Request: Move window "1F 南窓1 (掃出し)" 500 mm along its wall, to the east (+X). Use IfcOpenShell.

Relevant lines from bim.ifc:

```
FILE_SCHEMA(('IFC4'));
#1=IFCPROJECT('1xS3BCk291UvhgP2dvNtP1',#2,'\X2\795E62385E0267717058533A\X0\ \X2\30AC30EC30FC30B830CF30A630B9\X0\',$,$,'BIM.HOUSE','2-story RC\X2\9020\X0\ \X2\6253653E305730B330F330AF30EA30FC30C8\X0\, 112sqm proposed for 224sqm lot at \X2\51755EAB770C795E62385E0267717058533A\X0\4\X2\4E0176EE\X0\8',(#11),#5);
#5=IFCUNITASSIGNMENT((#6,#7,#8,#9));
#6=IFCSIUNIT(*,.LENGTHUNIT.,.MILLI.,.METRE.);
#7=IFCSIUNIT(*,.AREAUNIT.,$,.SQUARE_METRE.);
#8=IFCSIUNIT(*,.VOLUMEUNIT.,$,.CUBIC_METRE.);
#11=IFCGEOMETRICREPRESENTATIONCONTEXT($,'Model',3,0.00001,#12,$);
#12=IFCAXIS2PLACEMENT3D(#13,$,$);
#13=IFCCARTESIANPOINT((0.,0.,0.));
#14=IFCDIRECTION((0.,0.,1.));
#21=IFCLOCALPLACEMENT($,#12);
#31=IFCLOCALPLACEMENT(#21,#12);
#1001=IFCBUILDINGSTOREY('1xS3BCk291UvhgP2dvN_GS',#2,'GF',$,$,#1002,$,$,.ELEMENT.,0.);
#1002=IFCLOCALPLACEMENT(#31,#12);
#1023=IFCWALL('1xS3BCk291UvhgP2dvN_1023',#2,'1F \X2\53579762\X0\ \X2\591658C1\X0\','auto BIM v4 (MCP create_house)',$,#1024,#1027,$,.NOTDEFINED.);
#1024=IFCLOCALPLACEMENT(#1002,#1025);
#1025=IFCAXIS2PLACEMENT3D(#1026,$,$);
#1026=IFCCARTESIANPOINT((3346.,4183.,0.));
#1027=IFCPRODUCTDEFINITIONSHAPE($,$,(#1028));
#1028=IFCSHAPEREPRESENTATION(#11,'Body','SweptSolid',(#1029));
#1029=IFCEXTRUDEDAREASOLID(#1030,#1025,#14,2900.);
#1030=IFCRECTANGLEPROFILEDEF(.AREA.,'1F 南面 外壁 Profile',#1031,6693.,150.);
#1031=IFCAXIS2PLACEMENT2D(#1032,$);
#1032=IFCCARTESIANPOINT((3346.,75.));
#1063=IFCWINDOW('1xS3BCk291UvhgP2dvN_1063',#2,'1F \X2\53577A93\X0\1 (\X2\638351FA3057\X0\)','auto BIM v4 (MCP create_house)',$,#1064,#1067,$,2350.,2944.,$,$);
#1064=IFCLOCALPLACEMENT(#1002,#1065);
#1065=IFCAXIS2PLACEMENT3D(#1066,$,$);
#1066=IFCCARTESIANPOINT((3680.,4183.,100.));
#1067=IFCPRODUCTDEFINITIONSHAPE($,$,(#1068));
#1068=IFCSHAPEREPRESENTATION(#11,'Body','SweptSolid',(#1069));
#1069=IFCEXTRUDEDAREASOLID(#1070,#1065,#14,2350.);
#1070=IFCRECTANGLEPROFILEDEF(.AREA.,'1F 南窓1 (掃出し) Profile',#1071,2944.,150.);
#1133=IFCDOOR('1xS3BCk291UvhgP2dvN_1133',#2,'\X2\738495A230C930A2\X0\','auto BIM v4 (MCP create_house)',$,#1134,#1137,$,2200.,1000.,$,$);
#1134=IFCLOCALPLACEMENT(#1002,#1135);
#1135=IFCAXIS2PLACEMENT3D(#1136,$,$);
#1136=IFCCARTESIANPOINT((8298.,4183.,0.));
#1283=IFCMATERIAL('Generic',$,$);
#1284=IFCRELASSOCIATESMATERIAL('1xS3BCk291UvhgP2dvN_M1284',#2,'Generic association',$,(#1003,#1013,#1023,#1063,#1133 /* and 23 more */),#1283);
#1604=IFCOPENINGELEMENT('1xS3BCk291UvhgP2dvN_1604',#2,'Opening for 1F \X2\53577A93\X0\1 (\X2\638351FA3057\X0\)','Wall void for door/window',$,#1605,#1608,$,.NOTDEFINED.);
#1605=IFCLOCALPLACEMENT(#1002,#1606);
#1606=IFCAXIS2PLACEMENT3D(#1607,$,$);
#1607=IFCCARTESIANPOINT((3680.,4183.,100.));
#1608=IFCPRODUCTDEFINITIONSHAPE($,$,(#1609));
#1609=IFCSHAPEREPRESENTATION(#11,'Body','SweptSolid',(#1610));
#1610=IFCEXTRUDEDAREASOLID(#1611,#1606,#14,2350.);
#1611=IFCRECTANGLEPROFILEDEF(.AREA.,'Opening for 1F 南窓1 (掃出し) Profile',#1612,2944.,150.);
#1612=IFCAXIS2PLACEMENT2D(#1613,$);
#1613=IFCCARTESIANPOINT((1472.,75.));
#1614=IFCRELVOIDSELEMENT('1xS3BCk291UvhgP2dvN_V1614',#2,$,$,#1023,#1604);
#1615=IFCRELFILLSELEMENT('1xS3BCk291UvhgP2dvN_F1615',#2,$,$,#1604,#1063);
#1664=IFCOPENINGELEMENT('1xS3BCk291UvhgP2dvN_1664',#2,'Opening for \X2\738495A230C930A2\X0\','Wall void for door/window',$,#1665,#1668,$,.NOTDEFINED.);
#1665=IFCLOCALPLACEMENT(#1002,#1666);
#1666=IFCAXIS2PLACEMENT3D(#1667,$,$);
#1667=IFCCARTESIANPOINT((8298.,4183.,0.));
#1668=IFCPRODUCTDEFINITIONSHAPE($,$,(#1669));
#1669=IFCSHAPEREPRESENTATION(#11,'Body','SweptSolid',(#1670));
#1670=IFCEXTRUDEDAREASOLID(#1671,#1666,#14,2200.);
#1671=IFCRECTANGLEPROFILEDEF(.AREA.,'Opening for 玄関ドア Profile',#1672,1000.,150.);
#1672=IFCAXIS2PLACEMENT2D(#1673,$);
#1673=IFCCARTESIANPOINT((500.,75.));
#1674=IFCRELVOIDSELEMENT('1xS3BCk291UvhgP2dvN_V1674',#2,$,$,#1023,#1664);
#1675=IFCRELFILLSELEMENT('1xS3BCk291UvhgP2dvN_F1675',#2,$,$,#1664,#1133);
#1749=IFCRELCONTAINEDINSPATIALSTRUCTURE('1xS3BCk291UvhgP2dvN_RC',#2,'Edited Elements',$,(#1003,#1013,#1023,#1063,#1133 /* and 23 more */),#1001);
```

```python
import ifcopenshell
import ifcopenshell.api.geometry
import ifcopenshell.util.placement

model = ifcopenshell.open("bim.ifc")

window = model.by_guid("1xS3BCk291UvhgP2dvN_1063")
opening = window.FillsVoids[0].RelatingOpeningElement
wall = opening.VoidsElements[0].RelatingBuildingElement

wall_matrix = ifcopenshell.util.placement.get_local_placement(wall.ObjectPlacement)
shift = wall_matrix[:3, 0] * 500.0
before = ifcopenshell.util.placement.get_local_placement(window.ObjectPlacement)[:3, 3].copy()

# The window is not placed relative to its opening, so move both.
for product in (opening, window):
    matrix = ifcopenshell.util.placement.get_local_placement(product.ObjectPlacement)
    matrix[:3, 3] += shift
    ifcopenshell.api.geometry.edit_object_placement(model, product=product, matrix=matrix, is_si=False)

after = ifcopenshell.util.placement.get_local_placement(window.ObjectPlacement)[:3, 3]
print("window moved by", (after - before).round(3) + 0.0)

model.write("bim_rev.ifc")
```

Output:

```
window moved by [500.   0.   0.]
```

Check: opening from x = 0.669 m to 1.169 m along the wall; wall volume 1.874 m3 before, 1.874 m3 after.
